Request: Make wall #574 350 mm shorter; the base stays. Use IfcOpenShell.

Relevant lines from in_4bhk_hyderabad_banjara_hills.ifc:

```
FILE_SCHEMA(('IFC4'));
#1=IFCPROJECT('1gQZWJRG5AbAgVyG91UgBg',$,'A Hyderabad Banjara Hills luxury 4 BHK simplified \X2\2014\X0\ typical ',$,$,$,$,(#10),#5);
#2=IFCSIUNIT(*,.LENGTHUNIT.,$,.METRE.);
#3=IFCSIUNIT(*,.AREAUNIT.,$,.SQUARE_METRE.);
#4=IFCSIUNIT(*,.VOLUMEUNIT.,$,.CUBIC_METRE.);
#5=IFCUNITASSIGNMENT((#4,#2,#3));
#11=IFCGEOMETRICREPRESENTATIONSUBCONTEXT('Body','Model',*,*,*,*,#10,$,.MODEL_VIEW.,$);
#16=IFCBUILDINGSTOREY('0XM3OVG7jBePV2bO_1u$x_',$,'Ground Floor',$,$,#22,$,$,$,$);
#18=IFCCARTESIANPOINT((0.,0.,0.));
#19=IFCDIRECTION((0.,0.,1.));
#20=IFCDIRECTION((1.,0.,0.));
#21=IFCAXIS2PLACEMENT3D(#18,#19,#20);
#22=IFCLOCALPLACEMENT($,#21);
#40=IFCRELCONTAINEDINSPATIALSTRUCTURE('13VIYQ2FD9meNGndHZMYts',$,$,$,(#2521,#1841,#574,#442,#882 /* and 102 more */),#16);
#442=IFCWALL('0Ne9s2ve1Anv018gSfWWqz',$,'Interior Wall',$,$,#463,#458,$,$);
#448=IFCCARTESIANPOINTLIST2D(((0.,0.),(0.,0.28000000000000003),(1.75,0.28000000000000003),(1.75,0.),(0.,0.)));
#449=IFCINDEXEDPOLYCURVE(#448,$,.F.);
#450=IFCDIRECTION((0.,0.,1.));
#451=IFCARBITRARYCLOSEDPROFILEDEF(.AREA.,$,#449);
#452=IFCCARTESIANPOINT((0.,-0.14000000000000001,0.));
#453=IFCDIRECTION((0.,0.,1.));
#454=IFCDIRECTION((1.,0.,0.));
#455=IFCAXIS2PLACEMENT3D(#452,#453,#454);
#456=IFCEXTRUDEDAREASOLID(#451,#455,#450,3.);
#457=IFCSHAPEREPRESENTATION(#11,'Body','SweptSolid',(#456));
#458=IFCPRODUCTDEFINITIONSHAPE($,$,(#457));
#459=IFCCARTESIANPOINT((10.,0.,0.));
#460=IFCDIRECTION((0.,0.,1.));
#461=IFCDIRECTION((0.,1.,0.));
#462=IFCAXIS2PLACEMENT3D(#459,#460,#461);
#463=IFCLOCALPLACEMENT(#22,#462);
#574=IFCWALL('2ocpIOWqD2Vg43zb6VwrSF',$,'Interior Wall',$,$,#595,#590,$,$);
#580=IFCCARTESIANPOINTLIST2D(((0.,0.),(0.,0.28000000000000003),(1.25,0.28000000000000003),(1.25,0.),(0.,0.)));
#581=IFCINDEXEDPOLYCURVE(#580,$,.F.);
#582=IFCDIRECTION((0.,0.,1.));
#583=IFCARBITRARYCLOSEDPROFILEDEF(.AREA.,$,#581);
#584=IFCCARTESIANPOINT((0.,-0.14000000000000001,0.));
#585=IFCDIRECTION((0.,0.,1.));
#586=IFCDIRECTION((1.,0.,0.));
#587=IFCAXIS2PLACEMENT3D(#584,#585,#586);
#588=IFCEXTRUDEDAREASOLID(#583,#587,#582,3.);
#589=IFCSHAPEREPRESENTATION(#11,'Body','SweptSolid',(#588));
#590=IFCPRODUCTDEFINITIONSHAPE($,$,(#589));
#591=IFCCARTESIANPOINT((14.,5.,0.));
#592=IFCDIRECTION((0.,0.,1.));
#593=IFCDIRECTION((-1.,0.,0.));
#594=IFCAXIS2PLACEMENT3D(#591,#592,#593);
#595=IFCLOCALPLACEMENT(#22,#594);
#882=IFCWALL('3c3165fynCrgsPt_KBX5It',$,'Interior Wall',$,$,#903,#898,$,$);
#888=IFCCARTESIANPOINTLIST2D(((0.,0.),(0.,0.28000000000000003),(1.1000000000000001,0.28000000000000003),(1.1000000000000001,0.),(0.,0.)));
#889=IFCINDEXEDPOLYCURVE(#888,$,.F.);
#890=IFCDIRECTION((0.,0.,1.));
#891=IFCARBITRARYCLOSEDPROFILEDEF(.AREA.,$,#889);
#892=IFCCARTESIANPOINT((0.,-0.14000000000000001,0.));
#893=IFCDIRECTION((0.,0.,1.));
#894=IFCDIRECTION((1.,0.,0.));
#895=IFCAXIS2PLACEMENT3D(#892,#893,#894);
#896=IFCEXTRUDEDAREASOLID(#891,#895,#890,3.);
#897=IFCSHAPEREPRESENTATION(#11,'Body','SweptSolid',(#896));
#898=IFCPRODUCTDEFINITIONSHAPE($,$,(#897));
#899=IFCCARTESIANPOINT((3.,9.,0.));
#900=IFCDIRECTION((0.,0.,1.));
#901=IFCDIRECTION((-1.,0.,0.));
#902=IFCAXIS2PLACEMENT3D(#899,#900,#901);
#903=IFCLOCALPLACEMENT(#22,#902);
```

```python
import ifcopenshell
import ifcopenshell.geom
import ifcopenshell.util.representation
import ifcopenshell.util.shape
import ifcopenshell.util.unit

model = ifcopenshell.open("in_4bhk_hyderabad_banjara_hills.ifc")
unit_scale = ifcopenshell.util.unit.calculate_unit_scale(model)
settings = ifcopenshell.geom.settings()


def volume(element):
    """Net volume in cubic metres, openings subtracted."""
    shape = ifcopenshell.geom.create_shape(settings, element)
    return ifcopenshell.util.shape.get_volume(shape.geometry)


wall = model.by_guid("2ocpIOWqD2Vg43zb6VwrSF")
before = volume(wall)

body = ifcopenshell.util.representation.get_representation(wall, "Model", "Body")
solid = body.Items[0]
old_height = solid.Depth
solid.Depth -= 0.35 / unit_scale
after = volume(wall)

print(f"height {old_height:g} -> {solid.Depth:g}, volume {before:.3f} -> {after:.3f} m3")

model.write("in_4bhk_hyderabad_banjara_hills-out.ifc")
```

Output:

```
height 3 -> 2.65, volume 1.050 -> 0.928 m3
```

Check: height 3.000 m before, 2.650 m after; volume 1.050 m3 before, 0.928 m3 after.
